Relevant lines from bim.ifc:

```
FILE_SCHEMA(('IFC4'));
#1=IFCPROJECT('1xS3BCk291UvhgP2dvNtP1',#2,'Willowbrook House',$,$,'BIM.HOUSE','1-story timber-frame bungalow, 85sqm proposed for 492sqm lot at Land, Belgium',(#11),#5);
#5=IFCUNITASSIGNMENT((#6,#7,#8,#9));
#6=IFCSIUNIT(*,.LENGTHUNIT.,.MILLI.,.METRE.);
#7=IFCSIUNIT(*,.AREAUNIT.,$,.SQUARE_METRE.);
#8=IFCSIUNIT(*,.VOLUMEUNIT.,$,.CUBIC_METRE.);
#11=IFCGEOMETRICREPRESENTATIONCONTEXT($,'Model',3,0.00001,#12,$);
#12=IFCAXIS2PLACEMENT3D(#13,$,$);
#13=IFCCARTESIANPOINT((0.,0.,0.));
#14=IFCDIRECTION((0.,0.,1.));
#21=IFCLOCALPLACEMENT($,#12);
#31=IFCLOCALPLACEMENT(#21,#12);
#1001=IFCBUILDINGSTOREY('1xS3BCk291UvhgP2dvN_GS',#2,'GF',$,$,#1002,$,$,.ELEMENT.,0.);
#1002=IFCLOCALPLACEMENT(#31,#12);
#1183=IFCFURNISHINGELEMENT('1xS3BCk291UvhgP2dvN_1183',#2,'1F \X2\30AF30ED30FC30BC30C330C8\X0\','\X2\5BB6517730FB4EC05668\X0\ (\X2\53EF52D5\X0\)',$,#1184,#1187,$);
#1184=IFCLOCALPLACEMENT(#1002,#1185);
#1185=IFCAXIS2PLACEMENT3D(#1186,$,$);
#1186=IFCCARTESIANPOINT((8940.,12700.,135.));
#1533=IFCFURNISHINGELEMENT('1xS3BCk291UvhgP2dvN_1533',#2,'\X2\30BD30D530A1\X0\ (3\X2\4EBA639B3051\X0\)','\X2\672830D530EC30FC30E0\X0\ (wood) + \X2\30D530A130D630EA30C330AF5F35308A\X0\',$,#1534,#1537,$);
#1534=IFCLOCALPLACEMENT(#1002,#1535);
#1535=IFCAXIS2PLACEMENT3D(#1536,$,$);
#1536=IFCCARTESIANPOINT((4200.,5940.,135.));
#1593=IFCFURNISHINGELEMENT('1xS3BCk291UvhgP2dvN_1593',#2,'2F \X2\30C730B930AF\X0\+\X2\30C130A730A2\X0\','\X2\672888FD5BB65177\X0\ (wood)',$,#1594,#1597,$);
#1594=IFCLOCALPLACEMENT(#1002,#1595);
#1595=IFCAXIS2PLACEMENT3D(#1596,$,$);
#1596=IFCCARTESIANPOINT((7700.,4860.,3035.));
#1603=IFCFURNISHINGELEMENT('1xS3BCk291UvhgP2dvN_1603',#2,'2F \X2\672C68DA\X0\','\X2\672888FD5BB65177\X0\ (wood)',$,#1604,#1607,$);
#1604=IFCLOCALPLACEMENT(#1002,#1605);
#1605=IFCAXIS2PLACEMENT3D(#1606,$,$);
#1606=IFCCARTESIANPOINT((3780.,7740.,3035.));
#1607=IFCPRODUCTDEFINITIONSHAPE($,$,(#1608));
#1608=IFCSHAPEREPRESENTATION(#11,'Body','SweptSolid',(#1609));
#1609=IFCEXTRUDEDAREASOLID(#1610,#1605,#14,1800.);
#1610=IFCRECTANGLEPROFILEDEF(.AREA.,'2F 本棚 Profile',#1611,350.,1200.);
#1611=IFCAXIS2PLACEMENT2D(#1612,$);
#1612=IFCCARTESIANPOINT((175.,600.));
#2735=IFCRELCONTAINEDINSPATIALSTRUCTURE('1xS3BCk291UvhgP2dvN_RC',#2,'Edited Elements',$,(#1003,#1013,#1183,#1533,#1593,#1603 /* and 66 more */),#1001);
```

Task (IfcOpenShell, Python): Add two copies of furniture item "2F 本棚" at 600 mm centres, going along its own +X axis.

```python
import ifcopenshell
import ifcopenshell.api.geometry
import ifcopenshell.api.root
import ifcopenshell.util.element
import ifcopenshell.util.placement

model = ifcopenshell.open("bim.ifc")


def reuse_history(source, copy):
    """copy_class also copies each property set's owner history, people and application; keep the originals."""
    for rel in copy.IsDefinedBy:
        if rel.is_a("IfcRelDefinesByProperties") and (history := rel.RelatingPropertyDefinition.OwnerHistory):
            rel.RelatingPropertyDefinition.OwnerHistory = source.OwnerHistory
            ifcopenshell.util.element.remove_deep2(model, history)


source = model.by_id(1603)
base = ifcopenshell.util.placement.get_local_placement(source.ObjectPlacement)
step = base[:3, 0] * 600.0

for i in range(1, 3):
    copy = ifcopenshell.api.root.copy_class(model, product=source)
    copy.Representation = ifcopenshell.util.element.copy_deep(
        model, source.Representation, exclude=["IfcGeometricRepresentationContext", "IfcRepresentationMap"]
    )
    reuse_history(source, copy)
    matrix = base.copy()
    matrix[:3, 3] += i * step
    print("added at", matrix[:3, 3].round(3) + 0.0)
    ifcopenshell.api.geometry.edit_object_placement(model, product=copy, matrix=matrix, is_si=False)

model.write("bim-out.ifc")
```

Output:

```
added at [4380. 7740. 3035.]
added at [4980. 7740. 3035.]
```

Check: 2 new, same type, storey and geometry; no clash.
